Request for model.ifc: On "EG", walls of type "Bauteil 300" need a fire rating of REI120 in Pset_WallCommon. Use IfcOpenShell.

First a look at what the model holds.

```python
import ifcopenshell
import ifcopenshell.util.element

model = ifcopenshell.open("model.ifc")
print(model.schema)
storey = next(s for s in model.by_type("IfcBuildingStorey") if s.Name == "EG")
walls = [e for e in ifcopenshell.util.element.get_decomposition(storey) if e.is_a("IfcWall")]
seen = {}
for e in walls:
    element_type = ifcopenshell.util.element.get_type(e)
    key = (element_type.Name if element_type != e and element_type else None, ifcopenshell.util.element.get_pset(e, "Pset_WallCommon", "FireRating"))
    seen[key] = seen.get(key, 0) + 1
for (name, value), count in sorted(seen.items(), key=str):
    print(count, "x", name, "|", value)
```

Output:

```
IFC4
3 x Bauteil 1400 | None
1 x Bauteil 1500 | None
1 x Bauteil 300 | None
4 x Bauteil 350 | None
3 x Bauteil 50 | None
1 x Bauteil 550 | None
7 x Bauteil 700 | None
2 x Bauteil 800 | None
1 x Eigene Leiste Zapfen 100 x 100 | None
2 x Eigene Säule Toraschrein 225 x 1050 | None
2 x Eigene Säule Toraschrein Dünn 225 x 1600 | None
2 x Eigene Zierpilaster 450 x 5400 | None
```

```python
import ifcopenshell
import ifcopenshell.api.pset
import ifcopenshell.util.element

model = ifcopenshell.open("model.ifc")

storey = next(s for s in model.by_type("IfcBuildingStorey") if s.Name == "EG")
walls = [e for e in ifcopenshell.util.element.get_decomposition(storey) if e.is_a("IfcWall")]

count = 0
for e in walls:
    element_type = ifcopenshell.util.element.get_type(e)
    if element_type in (None, e) or element_type.Name != "Bauteil 300":
        continue
    # add_pset returns the element's existing set when there is one.
    pset = ifcopenshell.api.pset.add_pset(model, product=e, name="Pset_WallCommon")
    ifcopenshell.api.pset.edit_pset(model, pset=pset, properties={"FireRating": "REI120"})
    count += 1

print(count, "walls updated")

model.write("model_v2.ifc")
```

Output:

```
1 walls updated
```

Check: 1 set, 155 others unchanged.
